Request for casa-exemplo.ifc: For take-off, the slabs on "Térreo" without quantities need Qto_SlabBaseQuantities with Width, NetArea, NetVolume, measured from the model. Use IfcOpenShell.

First a look at what the model holds.

```python
import ifcopenshell
import ifcopenshell.util.element
import ifcopenshell.util.unit

model = ifcopenshell.open("casa-exemplo.ifc")
print(model.schema)
for unit_type in ("LENGTHUNIT", "AREAUNIT", "VOLUMEUNIT"):
    print(unit_type, ifcopenshell.util.unit.calculate_unit_scale(model, unit_type))
storey = next(s for s in model.by_type("IfcBuildingStorey") if s.Name == "Térreo")
slabs = [e for e in ifcopenshell.util.element.get_decomposition(storey) if e.is_a("IfcSlab")]
for e in sorted(slabs, key=lambda e: e.id()):
    print(e.id(), e.is_a(), e.Name, list(ifcopenshell.util.element.get_psets(e, qtos_only=True)), sep=" | ")
```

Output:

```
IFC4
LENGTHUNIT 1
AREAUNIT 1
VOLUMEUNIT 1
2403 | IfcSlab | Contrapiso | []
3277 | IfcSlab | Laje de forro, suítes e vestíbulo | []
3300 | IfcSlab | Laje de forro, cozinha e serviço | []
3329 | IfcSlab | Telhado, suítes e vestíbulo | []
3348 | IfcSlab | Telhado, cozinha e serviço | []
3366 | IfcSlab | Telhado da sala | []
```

```python
import ifcopenshell
import ifcopenshell.api.pset
import ifcopenshell.geom
import ifcopenshell.util.element
import ifcopenshell.util.shape
import ifcopenshell.util.unit

model = ifcopenshell.open("casa-exemplo.ifc")
unit_scale = ifcopenshell.util.unit.calculate_unit_scale(model)
area_scale = ifcopenshell.util.unit.calculate_unit_scale(model, "AREAUNIT")
volume_scale = ifcopenshell.util.unit.calculate_unit_scale(model, "VOLUMEUNIT")
settings = ifcopenshell.geom.settings()

storey = next(s for s in model.by_type("IfcBuildingStorey") if s.Name == "Térreo")
slabs = [e for e in ifcopenshell.util.element.get_decomposition(storey) if e.is_a("IfcSlab")]

for e in sorted(slabs, key=lambda e: e.id()):
    if ifcopenshell.util.element.get_psets(e, qtos_only=True, should_inherit=False):
        continue
    # Geometry comes back in metres, in the element's own axes.
    shape = ifcopenshell.geom.create_shape(settings, e)
    values = {
        "Width": ifcopenshell.util.shape.get_z(shape.geometry) / unit_scale,
        "NetArea": ifcopenshell.util.shape.get_footprint_area(shape.geometry) / area_scale,
        "NetVolume": ifcopenshell.util.shape.get_volume(shape.geometry) / volume_scale,
    }
    qto = ifcopenshell.api.pset.add_qto(model, product=e, name="Qto_SlabBaseQuantities")
    ifcopenshell.api.pset.edit_qto(model, qto=qto, properties=values)
    print(e.id(), {k: round(v, 3) for k, v in values.items()})

model.write("casa-exemplo-out.ifc")
```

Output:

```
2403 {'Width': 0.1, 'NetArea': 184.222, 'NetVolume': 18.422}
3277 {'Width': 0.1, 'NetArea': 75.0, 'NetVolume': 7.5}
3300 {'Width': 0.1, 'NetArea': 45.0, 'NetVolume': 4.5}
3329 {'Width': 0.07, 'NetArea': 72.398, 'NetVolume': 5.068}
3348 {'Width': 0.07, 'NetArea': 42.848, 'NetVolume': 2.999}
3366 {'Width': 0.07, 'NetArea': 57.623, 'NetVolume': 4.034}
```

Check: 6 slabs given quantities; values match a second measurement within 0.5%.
